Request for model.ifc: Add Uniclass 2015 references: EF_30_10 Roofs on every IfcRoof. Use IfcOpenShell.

First a look at what the model holds.

```python
import ifcopenshell

model = ifcopenshell.open("model.ifc")
print(model.schema)
print("classifications:", [c.Name for c in model.by_type("IfcClassification")])
for ifc_class in ("IfcDoor", "IfcRoof", "IfcStair", "IfcWall", "IfcWindow"):
    print(ifc_class, len(model.by_type(ifc_class)))
```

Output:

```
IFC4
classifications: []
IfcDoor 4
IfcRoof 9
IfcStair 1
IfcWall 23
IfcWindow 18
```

```python
import ifcopenshell
import ifcopenshell.api.classification

model = ifcopenshell.open("model.ifc")

system = ifcopenshell.api.classification.add_classification(model, classification="Uniclass 2015")

codes = {
    "IfcRoof": ("EF_30_10", "Roofs"),
}
for ifc_class, (code, name) in codes.items():
    products = model.by_type(ifc_class)
    ifcopenshell.api.classification.add_reference(
        model, products=products, classification=system, identification=code, name=name
    )
    print(code, len(products))

model.write("model_edited.ifc")
```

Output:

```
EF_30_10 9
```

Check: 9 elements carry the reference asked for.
